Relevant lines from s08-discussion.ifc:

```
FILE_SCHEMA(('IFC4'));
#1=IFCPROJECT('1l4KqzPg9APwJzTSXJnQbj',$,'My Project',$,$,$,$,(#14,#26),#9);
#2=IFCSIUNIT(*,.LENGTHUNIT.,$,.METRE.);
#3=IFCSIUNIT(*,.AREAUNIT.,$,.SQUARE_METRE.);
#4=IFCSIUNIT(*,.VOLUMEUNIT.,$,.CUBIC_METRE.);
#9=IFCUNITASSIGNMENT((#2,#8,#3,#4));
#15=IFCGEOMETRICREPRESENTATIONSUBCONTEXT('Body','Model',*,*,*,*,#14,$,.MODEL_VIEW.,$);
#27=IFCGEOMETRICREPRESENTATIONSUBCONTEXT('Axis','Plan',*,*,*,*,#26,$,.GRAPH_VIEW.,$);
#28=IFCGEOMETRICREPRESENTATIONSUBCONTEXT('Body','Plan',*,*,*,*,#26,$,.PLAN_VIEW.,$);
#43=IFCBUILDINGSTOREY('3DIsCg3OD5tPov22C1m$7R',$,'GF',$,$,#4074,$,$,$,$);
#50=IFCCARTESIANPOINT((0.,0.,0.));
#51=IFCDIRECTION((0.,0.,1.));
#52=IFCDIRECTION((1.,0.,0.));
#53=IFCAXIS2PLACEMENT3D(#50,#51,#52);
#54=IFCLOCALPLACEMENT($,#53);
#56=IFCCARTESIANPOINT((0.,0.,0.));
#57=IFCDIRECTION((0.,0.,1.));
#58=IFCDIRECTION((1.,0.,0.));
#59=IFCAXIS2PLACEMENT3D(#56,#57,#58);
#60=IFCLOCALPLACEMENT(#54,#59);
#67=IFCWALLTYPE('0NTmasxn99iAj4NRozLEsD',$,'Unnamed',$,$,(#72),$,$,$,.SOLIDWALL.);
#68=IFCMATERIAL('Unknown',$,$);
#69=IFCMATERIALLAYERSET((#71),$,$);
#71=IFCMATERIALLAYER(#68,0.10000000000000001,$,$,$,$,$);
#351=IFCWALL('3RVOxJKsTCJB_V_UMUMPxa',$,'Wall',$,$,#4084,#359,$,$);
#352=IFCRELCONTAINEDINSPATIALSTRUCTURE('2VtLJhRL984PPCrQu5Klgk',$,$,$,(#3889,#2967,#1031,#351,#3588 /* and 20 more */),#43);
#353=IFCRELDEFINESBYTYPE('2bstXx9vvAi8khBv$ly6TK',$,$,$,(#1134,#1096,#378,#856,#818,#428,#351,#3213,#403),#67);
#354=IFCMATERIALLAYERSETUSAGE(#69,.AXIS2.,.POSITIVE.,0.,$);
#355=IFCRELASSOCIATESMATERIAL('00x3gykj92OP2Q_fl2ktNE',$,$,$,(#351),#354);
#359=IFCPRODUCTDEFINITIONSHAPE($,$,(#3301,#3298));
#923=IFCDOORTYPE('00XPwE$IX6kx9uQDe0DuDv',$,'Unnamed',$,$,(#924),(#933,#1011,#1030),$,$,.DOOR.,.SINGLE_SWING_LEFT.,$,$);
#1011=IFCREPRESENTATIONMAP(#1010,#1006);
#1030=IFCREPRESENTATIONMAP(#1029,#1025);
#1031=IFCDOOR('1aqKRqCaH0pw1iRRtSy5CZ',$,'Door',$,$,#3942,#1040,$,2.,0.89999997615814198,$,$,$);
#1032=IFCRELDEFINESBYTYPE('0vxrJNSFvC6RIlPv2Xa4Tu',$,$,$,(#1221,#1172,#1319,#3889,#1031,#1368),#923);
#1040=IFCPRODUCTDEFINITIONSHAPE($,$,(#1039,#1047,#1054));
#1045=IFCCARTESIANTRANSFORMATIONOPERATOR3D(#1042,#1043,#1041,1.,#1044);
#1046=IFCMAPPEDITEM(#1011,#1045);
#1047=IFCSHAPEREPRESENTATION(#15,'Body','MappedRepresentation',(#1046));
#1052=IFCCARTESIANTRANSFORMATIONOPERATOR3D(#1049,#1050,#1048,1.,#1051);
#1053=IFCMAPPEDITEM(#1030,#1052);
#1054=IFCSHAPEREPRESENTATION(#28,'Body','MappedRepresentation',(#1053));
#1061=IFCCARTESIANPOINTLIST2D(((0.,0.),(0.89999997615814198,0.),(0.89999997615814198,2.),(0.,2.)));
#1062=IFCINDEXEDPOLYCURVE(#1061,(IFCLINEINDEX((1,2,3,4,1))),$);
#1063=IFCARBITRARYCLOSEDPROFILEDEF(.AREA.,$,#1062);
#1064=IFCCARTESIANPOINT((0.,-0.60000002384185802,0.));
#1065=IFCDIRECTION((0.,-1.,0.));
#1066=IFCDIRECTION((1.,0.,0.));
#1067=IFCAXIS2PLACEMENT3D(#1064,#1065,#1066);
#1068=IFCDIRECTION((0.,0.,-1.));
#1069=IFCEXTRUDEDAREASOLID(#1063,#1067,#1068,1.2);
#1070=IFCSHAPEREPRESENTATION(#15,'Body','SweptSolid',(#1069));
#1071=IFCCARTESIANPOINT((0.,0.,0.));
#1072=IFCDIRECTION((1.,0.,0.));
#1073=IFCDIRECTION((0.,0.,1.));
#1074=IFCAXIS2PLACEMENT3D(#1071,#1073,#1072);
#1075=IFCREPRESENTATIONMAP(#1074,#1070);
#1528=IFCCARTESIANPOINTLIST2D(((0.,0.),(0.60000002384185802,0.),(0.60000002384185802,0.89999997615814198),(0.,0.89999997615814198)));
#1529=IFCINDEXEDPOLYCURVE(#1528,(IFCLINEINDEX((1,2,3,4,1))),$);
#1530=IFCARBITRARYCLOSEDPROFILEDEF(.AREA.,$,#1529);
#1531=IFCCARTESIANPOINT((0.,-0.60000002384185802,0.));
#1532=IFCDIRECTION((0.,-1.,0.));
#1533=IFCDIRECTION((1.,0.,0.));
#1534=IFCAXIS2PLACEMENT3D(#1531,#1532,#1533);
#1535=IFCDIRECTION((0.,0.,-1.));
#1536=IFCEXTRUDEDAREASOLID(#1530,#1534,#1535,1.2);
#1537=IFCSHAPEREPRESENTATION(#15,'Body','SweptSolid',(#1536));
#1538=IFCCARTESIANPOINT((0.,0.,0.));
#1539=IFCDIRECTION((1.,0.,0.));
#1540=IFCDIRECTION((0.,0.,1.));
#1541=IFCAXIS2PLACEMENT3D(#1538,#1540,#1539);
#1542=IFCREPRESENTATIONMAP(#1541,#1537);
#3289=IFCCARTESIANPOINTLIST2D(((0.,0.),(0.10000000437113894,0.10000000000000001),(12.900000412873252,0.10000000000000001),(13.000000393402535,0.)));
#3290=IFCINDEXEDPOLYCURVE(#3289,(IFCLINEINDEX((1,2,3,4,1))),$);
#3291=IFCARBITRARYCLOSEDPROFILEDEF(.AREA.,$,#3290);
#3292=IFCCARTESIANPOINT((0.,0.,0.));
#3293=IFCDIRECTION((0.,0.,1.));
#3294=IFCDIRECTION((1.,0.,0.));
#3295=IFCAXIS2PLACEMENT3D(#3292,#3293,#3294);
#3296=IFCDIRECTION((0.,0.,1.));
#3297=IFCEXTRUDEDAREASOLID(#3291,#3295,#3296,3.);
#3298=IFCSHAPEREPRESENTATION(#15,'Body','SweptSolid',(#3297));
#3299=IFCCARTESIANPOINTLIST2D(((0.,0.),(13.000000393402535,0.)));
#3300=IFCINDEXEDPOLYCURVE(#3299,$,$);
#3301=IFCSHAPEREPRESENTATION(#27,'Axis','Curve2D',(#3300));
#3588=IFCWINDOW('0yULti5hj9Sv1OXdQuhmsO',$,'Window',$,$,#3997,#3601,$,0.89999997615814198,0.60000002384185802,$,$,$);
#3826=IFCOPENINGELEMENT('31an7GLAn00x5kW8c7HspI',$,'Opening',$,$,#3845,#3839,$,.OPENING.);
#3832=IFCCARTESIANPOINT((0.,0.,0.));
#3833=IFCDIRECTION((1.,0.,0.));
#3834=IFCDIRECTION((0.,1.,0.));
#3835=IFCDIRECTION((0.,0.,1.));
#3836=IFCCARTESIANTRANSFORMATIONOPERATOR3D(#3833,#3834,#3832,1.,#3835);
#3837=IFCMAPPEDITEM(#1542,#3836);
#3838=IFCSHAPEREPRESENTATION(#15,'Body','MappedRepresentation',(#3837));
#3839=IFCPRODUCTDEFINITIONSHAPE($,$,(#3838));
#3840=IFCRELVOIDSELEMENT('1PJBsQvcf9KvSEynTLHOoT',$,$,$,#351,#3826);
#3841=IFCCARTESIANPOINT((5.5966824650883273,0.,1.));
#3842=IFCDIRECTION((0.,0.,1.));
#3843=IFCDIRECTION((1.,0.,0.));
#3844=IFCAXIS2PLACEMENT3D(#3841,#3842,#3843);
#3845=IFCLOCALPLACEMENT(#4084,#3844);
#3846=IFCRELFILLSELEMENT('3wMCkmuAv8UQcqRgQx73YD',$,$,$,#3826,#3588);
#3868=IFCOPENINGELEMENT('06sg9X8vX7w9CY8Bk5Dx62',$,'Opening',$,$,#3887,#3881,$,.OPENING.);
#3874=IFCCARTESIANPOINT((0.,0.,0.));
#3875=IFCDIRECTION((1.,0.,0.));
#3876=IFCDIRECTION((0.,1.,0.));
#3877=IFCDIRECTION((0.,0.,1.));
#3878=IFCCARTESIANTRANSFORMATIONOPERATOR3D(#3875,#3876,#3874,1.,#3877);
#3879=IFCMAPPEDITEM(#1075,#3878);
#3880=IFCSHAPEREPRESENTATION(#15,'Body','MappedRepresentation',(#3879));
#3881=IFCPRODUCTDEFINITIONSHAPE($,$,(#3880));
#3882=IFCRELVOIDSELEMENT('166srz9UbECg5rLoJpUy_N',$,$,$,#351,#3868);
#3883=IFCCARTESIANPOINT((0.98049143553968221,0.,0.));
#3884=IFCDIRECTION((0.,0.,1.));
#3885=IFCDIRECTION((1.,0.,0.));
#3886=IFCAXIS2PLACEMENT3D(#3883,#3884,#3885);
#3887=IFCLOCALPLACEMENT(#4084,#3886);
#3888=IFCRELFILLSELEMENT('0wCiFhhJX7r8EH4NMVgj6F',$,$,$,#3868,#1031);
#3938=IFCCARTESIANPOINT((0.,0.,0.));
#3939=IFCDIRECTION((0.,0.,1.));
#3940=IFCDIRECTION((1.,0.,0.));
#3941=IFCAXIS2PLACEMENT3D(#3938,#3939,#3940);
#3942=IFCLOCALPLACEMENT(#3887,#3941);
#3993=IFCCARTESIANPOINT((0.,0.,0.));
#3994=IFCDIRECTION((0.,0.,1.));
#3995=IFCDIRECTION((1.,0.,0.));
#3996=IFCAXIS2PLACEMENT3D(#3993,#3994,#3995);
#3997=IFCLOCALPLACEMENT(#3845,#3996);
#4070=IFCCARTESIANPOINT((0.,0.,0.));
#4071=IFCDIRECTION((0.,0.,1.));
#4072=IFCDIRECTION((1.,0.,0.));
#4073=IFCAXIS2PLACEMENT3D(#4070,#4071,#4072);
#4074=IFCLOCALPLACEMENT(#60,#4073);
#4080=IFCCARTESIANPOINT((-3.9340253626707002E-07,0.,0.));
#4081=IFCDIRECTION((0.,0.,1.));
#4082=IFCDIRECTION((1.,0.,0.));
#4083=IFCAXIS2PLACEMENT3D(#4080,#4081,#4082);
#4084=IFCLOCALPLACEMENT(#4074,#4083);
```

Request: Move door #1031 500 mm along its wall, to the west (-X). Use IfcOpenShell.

```python
import ifcopenshell
import ifcopenshell.api.geometry
import ifcopenshell.util.placement
import ifcopenshell.util.unit

model = ifcopenshell.open("s08-discussion.ifc")
unit_scale = ifcopenshell.util.unit.calculate_unit_scale(model)

door = model.by_guid("1aqKRqCaH0pw1iRRtSy5CZ")
opening = door.FillsVoids[0].RelatingOpeningElement
wall = opening.VoidsElements[0].RelatingBuildingElement

wall_matrix = ifcopenshell.util.placement.get_local_placement(wall.ObjectPlacement)
shift = wall_matrix[:3, 0] * -0.5 / unit_scale
before = ifcopenshell.util.placement.get_local_placement(door.ObjectPlacement)[:3, 3].copy()

# The door is placed relative to its opening, so it follows when the opening moves.
matrix = ifcopenshell.util.placement.get_local_placement(opening.ObjectPlacement)
matrix[:3, 3] += shift
ifcopenshell.api.geometry.edit_object_placement(
    model, product=opening, matrix=matrix, is_si=False, should_transform_children=True
)

after = ifcopenshell.util.placement.get_local_placement(door.ObjectPlacement)[:3, 3]
print("door moved by", (after - before).round(3) + 0.0)

model.write("s08-discussion_updated.ifc")
```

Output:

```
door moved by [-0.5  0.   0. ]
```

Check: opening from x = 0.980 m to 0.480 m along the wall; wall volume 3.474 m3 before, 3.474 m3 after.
